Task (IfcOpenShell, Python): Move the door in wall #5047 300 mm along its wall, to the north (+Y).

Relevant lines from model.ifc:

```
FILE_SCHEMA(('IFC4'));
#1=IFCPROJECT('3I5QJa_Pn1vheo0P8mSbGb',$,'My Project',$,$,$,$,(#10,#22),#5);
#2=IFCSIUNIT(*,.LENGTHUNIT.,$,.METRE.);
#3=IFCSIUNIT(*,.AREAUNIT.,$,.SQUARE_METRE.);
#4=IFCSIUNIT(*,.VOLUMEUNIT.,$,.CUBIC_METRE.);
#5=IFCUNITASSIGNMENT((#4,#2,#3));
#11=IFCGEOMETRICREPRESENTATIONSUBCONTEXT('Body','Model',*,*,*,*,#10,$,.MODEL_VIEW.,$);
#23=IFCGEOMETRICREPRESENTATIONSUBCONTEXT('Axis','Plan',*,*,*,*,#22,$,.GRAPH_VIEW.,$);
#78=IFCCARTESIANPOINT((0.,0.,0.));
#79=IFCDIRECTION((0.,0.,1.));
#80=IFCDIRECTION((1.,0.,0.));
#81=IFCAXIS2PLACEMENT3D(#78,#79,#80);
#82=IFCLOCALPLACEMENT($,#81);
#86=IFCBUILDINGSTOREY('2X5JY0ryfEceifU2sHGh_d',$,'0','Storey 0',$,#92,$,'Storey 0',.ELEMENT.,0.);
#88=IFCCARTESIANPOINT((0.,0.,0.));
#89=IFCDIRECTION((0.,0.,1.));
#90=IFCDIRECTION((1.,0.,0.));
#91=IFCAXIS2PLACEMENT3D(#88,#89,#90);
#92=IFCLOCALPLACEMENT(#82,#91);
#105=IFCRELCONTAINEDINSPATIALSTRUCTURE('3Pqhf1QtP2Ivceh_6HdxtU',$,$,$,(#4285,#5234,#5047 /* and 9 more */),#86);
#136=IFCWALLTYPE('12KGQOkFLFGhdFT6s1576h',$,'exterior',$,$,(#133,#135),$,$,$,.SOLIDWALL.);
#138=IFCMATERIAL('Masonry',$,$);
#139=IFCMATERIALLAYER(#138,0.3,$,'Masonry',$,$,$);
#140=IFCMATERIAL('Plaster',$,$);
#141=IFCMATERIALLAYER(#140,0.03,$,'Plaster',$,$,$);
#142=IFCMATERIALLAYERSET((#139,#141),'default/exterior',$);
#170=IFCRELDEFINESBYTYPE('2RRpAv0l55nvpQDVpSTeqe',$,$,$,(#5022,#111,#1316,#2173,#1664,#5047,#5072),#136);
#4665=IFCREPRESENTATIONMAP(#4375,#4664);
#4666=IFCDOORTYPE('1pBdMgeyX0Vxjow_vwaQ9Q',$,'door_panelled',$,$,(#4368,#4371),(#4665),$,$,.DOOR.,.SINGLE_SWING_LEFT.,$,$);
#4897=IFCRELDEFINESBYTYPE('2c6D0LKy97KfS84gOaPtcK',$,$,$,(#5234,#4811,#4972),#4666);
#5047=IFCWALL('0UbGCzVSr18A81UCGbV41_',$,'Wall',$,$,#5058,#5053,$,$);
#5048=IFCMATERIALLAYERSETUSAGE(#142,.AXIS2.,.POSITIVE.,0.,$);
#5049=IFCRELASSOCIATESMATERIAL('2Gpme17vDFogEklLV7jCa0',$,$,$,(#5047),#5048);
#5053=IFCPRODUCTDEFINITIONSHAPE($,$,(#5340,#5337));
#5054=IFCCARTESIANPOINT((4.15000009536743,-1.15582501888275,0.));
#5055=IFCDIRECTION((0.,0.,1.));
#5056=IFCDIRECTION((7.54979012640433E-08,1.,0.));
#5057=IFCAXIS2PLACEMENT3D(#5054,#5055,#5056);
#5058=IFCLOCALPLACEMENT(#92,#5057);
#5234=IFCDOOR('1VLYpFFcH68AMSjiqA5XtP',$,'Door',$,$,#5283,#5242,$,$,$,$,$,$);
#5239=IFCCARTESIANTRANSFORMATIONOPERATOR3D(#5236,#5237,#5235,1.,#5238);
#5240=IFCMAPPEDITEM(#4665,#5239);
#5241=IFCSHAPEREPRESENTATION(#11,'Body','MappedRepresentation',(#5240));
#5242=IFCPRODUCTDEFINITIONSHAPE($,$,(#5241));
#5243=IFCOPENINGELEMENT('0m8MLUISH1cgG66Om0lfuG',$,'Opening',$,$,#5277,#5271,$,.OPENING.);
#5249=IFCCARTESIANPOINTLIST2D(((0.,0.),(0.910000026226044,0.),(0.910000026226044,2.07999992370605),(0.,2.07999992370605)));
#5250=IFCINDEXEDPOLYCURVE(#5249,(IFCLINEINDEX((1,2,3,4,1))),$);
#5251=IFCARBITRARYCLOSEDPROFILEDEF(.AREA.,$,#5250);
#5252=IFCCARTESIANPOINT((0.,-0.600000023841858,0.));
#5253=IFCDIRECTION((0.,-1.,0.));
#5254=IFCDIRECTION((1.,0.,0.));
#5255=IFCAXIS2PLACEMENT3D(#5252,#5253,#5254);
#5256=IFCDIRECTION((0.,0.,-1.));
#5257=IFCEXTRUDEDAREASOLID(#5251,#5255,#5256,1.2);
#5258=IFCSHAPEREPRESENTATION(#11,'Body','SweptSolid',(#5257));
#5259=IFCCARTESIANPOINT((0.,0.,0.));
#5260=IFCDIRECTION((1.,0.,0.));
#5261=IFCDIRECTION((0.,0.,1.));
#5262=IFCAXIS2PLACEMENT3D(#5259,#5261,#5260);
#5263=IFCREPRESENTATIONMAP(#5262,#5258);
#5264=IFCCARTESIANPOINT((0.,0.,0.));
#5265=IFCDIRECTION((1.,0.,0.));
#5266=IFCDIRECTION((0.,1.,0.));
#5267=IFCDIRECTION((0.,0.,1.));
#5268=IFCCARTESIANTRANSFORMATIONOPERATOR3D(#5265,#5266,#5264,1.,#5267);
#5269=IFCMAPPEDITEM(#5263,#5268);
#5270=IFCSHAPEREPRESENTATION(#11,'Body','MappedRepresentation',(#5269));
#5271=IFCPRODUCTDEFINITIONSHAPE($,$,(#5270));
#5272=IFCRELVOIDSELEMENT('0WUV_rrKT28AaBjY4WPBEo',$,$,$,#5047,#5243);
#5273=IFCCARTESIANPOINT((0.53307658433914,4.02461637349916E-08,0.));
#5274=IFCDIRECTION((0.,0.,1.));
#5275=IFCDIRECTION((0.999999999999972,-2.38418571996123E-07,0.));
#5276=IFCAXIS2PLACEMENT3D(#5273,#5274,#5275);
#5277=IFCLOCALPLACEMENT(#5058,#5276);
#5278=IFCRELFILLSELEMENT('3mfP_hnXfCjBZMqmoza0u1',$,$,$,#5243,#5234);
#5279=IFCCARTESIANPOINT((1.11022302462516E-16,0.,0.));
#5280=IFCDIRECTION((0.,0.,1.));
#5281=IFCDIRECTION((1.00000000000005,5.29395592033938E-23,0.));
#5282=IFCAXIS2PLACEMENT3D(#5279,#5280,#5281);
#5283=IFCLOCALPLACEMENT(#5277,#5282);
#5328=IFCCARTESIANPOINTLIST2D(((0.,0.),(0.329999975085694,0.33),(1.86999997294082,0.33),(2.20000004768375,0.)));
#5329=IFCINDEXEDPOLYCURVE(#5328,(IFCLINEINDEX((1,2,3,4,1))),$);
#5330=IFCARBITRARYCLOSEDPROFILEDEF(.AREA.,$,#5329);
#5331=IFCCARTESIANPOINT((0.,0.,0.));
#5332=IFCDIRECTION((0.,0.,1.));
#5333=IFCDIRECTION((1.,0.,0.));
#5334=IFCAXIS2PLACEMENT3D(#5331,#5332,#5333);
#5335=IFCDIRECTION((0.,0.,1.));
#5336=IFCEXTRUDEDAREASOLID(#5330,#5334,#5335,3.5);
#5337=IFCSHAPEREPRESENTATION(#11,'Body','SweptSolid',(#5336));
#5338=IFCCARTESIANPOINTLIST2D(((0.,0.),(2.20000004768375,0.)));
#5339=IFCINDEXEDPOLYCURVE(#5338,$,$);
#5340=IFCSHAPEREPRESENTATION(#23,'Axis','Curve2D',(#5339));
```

```python
import ifcopenshell
import ifcopenshell.api.geometry
import ifcopenshell.util.placement

model = ifcopenshell.open("model.ifc")

door = model.by_guid("1VLYpFFcH68AMSjiqA5XtP")
opening = door.FillsVoids[0].RelatingOpeningElement
wall = opening.VoidsElements[0].RelatingBuildingElement

wall_matrix = ifcopenshell.util.placement.get_local_placement(wall.ObjectPlacement)
shift = wall_matrix[:3, 0] * 0.3
before = ifcopenshell.util.placement.get_local_placement(door.ObjectPlacement)[:3, 3].copy()

# The door is placed relative to its opening, so it follows when the opening moves.
matrix = ifcopenshell.util.placement.get_local_placement(opening.ObjectPlacement)
matrix[:3, 3] += shift
ifcopenshell.api.geometry.edit_object_placement(
    model, product=opening, matrix=matrix, is_si=False, should_transform_children=True
)

after = ifcopenshell.util.placement.get_local_placement(door.ObjectPlacement)[:3, 3]
print("door moved by", (after - before).round(3) + 0.0)

model.write("model-out.ifc")
```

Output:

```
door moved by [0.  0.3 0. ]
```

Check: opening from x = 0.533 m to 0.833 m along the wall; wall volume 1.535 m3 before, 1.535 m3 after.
